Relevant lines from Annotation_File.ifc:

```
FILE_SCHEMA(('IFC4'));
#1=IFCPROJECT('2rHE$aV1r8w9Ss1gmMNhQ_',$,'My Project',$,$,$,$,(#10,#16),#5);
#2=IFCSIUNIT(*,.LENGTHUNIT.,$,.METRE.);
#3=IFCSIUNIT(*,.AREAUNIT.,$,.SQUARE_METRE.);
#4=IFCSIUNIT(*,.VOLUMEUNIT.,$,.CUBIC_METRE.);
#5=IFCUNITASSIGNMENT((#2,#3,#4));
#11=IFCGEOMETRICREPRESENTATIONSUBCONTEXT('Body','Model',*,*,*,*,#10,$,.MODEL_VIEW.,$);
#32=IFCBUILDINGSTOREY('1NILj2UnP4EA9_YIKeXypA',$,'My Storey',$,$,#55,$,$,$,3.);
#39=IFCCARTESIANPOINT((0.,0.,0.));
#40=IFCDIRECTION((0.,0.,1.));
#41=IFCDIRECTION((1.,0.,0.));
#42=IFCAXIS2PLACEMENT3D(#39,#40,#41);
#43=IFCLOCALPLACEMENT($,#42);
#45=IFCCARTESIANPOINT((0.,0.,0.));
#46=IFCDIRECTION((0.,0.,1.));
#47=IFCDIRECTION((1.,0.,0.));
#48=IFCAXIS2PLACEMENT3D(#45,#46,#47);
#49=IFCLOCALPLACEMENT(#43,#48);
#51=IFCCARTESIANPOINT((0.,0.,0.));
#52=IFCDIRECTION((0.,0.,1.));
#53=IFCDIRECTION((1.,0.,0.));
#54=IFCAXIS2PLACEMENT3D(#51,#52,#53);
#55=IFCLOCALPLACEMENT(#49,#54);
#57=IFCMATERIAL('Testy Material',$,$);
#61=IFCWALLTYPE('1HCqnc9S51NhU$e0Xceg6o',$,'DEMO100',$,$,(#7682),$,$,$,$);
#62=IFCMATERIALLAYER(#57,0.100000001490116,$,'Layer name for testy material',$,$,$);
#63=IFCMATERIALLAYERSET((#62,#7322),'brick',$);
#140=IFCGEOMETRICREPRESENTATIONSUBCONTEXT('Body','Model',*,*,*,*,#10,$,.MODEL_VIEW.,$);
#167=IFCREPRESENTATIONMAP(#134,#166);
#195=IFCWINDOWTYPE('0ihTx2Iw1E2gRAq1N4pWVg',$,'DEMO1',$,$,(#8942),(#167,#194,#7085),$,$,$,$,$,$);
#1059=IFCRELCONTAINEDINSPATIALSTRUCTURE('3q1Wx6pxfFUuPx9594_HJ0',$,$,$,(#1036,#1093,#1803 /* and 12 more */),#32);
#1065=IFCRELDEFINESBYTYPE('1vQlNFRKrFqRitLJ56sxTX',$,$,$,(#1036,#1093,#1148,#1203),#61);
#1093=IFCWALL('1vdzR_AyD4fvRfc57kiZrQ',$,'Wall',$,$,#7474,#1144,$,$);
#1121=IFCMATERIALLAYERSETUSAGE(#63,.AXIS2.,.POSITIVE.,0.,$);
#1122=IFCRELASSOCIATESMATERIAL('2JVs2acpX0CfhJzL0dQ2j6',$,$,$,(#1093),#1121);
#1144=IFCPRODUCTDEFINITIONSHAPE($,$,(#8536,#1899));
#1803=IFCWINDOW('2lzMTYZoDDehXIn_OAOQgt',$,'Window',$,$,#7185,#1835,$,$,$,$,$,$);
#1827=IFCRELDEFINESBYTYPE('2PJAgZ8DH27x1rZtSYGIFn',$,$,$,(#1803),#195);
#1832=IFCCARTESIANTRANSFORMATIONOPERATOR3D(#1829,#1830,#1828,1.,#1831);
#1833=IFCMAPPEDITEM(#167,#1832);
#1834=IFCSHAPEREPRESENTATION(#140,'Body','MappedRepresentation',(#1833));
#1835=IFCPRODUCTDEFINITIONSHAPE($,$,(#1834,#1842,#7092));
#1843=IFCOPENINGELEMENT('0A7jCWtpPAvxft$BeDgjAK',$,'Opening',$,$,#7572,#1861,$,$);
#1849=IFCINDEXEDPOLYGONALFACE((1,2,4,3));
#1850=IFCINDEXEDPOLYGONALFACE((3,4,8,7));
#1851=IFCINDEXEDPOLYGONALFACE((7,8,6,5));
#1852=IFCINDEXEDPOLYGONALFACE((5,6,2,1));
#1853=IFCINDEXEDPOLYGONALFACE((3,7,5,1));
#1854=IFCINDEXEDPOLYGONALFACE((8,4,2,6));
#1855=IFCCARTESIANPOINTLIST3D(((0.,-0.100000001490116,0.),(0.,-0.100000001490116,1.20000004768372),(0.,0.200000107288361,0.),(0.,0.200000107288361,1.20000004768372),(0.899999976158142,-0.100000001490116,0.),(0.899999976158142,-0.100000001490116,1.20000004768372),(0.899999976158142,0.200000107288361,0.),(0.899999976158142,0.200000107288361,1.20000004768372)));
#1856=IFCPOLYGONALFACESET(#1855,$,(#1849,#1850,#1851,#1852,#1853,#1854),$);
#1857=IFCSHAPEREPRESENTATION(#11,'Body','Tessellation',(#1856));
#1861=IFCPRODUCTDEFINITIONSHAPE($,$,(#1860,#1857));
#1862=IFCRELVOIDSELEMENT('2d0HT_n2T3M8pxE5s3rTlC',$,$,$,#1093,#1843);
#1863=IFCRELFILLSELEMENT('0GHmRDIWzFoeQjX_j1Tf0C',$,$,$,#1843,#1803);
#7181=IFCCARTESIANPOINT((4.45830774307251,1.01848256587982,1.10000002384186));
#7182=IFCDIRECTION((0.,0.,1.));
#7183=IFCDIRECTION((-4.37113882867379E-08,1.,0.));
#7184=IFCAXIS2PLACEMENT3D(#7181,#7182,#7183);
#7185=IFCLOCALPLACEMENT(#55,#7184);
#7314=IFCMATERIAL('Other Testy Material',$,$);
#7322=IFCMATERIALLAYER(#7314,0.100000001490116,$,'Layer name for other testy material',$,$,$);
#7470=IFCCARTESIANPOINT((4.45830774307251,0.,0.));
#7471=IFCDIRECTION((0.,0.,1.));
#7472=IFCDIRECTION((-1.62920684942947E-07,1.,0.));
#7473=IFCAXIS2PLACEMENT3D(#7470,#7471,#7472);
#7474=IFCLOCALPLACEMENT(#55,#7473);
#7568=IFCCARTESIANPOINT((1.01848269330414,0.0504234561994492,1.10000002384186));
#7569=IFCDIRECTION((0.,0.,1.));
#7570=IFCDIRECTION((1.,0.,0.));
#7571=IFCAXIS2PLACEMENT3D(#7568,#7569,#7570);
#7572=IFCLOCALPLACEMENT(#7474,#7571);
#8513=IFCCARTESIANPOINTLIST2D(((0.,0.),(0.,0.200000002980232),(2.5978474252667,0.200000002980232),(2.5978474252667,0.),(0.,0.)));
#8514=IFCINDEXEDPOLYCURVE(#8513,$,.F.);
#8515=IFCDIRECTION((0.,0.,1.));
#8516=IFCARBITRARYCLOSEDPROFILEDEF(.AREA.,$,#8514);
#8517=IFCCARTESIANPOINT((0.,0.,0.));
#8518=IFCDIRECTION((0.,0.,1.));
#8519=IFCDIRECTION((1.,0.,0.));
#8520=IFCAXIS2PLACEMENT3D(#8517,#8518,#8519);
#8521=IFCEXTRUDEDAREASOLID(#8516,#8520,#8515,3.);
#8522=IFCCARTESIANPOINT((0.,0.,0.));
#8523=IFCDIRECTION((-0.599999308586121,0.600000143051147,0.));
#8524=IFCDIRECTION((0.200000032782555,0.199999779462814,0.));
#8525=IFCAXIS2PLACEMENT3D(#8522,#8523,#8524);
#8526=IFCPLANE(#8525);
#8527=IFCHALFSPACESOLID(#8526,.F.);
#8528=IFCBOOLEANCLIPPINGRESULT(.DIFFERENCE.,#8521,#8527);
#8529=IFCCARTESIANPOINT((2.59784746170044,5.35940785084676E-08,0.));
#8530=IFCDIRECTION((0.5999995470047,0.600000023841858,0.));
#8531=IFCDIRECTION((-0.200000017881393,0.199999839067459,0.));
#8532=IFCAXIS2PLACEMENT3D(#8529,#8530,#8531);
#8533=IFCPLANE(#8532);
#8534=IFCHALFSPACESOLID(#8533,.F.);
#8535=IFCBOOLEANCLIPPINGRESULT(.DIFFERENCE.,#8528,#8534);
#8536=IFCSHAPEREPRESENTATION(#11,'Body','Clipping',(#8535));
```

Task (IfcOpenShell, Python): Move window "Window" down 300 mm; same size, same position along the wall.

```python
import numpy as np
import ifcopenshell
import ifcopenshell.api.geometry
import ifcopenshell.util.placement
import ifcopenshell.util.unit

model = ifcopenshell.open("Annotation_File.ifc")
unit_scale = ifcopenshell.util.unit.calculate_unit_scale(model)

window = model.by_guid("2lzMTYZoDDehXIn_OAOQgt")
opening = window.FillsVoids[0].RelatingOpeningElement
dz = -0.3 / unit_scale

shift = np.array([0.0, 0.0, dz])
# The window is not placed relative to its opening, so move both.
for product in (opening, window):
    matrix = ifcopenshell.util.placement.get_local_placement(product.ObjectPlacement)
    matrix[:3, 3] += shift
    ifcopenshell.api.geometry.edit_object_placement(model, product=product, matrix=matrix, is_si=False)

print(f"moved by {dz * unit_scale:+.3f} m")

model.write("Annotation_File-out.ifc")
```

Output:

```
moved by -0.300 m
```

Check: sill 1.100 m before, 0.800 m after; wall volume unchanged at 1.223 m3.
